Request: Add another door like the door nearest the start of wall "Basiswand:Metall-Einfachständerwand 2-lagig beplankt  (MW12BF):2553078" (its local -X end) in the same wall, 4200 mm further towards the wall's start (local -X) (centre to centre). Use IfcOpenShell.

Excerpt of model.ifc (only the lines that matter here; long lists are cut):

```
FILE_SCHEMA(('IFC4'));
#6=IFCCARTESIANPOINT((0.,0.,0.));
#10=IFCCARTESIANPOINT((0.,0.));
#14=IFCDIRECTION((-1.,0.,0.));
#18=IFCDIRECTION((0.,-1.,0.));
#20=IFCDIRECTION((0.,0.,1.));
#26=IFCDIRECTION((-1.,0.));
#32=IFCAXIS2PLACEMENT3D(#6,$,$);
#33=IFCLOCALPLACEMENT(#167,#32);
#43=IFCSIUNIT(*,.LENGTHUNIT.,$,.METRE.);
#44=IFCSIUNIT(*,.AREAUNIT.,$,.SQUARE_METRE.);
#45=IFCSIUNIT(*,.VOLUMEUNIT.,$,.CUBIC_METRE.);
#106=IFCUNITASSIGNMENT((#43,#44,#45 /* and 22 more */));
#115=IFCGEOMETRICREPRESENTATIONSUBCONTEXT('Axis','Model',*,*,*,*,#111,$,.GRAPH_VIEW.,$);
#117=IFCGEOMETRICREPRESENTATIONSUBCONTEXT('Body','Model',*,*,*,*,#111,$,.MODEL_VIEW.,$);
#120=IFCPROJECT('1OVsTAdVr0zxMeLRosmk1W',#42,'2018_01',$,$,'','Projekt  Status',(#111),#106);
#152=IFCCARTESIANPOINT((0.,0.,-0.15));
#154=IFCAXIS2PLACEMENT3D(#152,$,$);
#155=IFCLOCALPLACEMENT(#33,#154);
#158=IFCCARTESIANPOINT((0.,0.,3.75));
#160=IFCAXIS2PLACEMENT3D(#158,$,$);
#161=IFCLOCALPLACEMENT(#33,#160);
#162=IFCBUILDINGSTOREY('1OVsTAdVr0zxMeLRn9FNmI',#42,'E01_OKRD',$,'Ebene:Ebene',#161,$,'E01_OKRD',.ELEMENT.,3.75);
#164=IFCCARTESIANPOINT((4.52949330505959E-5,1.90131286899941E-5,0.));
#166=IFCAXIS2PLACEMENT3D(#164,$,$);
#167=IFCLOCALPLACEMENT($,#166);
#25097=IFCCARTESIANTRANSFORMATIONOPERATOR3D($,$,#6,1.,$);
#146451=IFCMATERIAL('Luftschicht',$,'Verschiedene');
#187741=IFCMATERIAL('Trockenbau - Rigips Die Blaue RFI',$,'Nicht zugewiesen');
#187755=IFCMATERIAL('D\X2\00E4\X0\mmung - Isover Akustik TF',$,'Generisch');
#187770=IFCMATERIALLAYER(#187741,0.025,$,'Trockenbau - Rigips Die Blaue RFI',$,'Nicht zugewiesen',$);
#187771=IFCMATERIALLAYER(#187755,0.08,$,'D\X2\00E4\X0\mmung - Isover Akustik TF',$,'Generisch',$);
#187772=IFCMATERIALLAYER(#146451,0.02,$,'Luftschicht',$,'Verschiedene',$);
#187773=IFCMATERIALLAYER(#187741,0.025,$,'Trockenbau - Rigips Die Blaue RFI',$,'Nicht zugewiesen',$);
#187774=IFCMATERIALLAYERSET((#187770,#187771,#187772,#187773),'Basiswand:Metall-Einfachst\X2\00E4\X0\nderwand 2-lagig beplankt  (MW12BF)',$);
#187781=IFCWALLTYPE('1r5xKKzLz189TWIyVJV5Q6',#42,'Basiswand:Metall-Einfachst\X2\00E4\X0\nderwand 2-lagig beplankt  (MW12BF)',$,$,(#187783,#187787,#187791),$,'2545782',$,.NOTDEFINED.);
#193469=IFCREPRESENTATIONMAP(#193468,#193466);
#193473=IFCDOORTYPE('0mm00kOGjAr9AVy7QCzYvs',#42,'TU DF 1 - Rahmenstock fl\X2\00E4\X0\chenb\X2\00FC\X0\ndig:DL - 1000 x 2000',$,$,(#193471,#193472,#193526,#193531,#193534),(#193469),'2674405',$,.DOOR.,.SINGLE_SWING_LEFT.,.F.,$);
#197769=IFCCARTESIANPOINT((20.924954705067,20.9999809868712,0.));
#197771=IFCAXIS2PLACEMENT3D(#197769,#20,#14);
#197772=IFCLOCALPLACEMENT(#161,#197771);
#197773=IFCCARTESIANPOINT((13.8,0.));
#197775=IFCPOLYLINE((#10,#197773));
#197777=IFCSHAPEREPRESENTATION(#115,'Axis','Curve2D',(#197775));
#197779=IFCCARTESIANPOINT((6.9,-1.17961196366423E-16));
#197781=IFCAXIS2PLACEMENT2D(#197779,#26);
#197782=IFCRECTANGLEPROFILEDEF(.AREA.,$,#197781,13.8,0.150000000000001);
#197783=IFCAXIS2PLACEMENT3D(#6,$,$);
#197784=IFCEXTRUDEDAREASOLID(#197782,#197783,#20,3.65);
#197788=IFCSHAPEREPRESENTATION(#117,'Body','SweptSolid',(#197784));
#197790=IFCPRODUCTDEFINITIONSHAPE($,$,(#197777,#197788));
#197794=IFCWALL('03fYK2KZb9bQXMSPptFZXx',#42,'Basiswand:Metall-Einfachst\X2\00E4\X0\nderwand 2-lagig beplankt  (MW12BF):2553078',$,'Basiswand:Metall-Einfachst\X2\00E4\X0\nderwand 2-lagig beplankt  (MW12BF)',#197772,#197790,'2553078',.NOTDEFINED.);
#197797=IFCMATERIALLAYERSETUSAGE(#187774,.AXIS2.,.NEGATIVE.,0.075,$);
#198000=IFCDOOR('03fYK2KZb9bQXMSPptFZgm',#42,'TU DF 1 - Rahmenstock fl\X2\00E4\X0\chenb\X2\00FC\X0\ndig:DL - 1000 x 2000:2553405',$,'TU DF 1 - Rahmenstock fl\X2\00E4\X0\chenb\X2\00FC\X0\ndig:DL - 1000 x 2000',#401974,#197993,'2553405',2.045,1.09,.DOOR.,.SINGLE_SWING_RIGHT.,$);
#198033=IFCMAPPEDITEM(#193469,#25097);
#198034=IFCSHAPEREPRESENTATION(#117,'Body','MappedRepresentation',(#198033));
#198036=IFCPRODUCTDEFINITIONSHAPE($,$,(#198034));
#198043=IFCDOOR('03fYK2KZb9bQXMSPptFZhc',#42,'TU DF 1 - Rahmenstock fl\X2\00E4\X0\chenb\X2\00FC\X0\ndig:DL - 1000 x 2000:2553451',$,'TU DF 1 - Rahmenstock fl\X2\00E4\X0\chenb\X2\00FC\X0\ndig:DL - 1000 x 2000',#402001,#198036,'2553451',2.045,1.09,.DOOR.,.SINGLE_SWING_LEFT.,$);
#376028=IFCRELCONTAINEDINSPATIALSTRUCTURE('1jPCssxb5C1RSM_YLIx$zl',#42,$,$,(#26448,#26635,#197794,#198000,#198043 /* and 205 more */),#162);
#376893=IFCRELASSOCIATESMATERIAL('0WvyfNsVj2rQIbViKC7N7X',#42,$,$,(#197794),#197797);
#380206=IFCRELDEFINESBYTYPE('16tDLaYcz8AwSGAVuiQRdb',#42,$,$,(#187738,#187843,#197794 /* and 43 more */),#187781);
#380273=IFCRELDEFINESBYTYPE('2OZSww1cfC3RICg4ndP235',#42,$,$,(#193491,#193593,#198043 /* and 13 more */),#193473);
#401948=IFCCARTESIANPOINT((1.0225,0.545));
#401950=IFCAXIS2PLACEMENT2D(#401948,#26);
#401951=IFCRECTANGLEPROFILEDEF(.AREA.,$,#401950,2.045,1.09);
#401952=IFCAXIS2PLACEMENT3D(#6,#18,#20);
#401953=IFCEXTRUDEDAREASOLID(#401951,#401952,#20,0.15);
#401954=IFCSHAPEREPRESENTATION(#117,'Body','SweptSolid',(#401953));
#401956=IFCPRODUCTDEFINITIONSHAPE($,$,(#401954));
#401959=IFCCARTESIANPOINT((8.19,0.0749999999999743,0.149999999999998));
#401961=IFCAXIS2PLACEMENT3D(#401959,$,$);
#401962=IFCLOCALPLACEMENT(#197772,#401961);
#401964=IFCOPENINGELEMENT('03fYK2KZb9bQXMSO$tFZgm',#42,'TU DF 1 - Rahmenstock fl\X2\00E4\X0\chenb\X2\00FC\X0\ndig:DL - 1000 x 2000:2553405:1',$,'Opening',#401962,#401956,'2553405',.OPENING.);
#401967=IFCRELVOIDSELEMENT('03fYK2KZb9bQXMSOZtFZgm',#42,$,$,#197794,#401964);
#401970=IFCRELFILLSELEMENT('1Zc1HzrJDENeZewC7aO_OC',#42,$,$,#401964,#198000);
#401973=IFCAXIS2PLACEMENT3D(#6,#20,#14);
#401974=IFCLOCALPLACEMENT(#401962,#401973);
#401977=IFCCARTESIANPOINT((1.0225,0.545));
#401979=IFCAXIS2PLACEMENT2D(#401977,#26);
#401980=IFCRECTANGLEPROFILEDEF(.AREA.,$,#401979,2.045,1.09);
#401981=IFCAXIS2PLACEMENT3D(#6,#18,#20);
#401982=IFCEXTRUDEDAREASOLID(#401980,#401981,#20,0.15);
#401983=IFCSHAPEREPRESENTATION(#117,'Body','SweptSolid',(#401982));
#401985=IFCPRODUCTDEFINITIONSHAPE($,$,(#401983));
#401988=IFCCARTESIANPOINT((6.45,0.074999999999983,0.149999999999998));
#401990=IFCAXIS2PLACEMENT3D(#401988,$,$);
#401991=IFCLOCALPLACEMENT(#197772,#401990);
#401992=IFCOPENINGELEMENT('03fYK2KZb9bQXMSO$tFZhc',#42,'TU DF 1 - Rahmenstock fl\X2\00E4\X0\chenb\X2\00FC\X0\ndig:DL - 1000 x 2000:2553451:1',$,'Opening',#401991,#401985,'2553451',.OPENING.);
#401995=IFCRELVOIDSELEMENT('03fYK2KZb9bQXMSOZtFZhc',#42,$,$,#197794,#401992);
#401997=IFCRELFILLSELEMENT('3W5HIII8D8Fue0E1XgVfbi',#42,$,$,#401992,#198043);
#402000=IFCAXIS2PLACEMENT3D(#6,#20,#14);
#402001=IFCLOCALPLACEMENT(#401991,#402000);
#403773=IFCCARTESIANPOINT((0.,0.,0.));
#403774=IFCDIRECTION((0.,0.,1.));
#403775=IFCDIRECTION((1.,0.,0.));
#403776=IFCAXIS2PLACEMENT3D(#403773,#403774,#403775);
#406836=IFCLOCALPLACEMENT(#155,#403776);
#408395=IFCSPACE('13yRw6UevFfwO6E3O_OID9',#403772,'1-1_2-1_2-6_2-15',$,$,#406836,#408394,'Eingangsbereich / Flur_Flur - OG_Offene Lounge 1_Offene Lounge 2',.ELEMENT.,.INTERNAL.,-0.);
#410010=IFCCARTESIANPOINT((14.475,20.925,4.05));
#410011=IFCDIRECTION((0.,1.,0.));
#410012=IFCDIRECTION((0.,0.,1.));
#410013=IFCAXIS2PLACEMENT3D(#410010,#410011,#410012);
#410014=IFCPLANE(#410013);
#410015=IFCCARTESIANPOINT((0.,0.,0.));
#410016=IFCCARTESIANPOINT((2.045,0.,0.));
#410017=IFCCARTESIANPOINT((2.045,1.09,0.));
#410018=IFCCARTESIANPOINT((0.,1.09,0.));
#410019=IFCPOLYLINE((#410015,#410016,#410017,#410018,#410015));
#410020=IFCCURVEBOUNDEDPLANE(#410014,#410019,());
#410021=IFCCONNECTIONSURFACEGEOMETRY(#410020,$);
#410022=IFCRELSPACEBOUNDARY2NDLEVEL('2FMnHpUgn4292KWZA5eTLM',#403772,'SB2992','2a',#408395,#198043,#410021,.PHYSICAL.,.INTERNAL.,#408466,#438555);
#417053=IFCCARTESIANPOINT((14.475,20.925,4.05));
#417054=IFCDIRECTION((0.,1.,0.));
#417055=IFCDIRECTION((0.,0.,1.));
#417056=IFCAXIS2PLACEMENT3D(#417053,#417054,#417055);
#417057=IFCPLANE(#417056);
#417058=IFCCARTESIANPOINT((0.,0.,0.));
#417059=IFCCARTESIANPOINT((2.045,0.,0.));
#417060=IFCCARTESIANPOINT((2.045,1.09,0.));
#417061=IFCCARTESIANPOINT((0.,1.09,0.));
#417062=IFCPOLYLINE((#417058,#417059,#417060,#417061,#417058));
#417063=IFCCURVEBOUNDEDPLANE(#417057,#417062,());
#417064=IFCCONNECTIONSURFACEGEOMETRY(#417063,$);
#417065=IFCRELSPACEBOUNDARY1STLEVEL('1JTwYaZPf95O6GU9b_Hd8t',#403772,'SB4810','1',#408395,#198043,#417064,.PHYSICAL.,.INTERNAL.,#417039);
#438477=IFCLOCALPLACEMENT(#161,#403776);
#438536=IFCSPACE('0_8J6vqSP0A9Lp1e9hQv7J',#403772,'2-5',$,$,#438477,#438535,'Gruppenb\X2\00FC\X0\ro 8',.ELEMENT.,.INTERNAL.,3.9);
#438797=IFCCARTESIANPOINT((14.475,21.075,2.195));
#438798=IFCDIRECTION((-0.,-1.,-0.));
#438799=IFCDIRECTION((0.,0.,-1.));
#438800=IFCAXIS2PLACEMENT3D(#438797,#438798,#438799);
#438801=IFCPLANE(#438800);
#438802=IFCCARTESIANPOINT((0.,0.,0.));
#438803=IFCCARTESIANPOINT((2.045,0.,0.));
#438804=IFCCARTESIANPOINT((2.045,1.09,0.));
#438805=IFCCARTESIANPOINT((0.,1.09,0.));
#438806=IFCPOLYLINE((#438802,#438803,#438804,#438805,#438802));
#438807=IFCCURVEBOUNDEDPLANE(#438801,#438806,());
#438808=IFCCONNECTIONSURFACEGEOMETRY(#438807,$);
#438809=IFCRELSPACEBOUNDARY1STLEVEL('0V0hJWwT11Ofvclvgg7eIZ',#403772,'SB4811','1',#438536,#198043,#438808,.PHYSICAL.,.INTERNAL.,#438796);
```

```python
import numpy as np
import ifcopenshell
import ifcopenshell.api.feature
import ifcopenshell.api.geometry
import ifcopenshell.api.root
import ifcopenshell.geom
import ifcopenshell.util.element
import ifcopenshell.util.placement
import ifcopenshell.util.shape
import ifcopenshell.util.unit

model = ifcopenshell.open("model.ifc")
unit_scale = ifcopenshell.util.unit.calculate_unit_scale(model)
settings = ifcopenshell.geom.settings()


def volume(element):
    """Net volume in cubic metres, openings subtracted."""
    shape = ifcopenshell.geom.create_shape(settings, element)
    return ifcopenshell.util.shape.get_volume(shape.geometry)


def reuse_history(source, copy):
    """copy_class also copies each property set's owner history, people and application; keep the originals."""
    for rel in copy.IsDefinedBy:
        if rel.is_a("IfcRelDefinesByProperties") and (history := rel.RelatingPropertyDefinition.OwnerHistory):
            rel.RelatingPropertyDefinition.OwnerHistory = source.OwnerHistory
            ifcopenshell.util.element.remove_deep2(model, history)


door = model.by_id(198043)
opening = door.FillsVoids[0].RelatingOpeningElement
wall = opening.VoidsElements[0].RelatingBuildingElement
before = volume(wall)
shift = ifcopenshell.util.placement.get_local_placement(wall.ObjectPlacement)[:3, 0] * -4.2 / unit_scale

# copy_class copies the void relationship, type, container and properties, but no geometry.
new_opening = ifcopenshell.api.root.copy_class(model, product=opening)
new_opening.Representation = ifcopenshell.util.element.copy_deep(
    model, opening.Representation, exclude=["IfcGeometricRepresentationContext", "IfcRepresentationMap"]
)
new_opening.Name = "TU DF 1 - Rahmenstock flächenbündig:DL - 1000 x 2000"
new_opening.Tag = None
new_door = ifcopenshell.api.root.copy_class(model, product=door)
new_door.Representation = ifcopenshell.util.element.copy_deep(
    model, door.Representation, exclude=["IfcGeometricRepresentationContext", "IfcRepresentationMap"]
)
new_door.Name = "TU DF 1 - Rahmenstock flächenbündig:DL - 1000 x 2000"
new_door.Tag = None
reuse_history(door, new_door)
ifcopenshell.api.feature.add_filling(model, opening=new_opening, element=new_door)

for old, new in ((opening, new_opening), (door, new_door)):
    matrix = ifcopenshell.util.placement.get_local_placement(old.ObjectPlacement)
    matrix[:3, 3] += shift
    ifcopenshell.api.geometry.edit_object_placement(model, product=new, matrix=matrix, is_si=False)

# The copied space boundaries still share their surfaces with the original.
for rel in new_door.ProvidesBoundaries:
    if rel.ConnectionGeometry:
        rel.ConnectionGeometry = ifcopenshell.util.element.copy_deep(model, rel.ConnectionGeometry)

# Space boundary surfaces are stored in each space's coordinates; move them too.
for rel in new_door.ProvidesBoundaries:
    if not rel.ConnectionGeometry:
        continue
    surface = rel.ConnectionGeometry.SurfaceOnRelatingElement.BasisSurface
    space_matrix = ifcopenshell.util.placement.get_local_placement(rel.RelatingSpace.ObjectPlacement)
    point = np.array(surface.Position.Location.Coordinates) + space_matrix[:3, :3].T @ shift
    surface.Position = model.createIfcAxis2Placement3D(
        model.createIfcCartesianPoint(point.tolist()), surface.Position.Axis, surface.Position.RefDirection
    )

after = volume(wall)

print(f"wall volume {before:.3f} -> {after:.3f} m3")

model.write("model-out.ifc")
```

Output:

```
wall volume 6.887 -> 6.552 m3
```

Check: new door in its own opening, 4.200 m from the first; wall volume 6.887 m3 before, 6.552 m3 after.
